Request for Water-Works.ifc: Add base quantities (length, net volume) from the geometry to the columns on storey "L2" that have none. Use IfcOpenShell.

First a look at what the model holds.

```python
import ifcopenshell
import ifcopenshell.util.element
import ifcopenshell.util.unit

model = ifcopenshell.open("Water-Works.ifc")
print(model.schema)
for unit_type in ("LENGTHUNIT", "AREAUNIT", "VOLUMEUNIT"):
    print(unit_type, ifcopenshell.util.unit.calculate_unit_scale(model, unit_type))
storey = next(s for s in model.by_type("IfcBuildingStorey") if s.Name == "L2")
columns = [e for e in ifcopenshell.util.element.get_decomposition(storey) if e.is_a("IfcColumn")]
for e in sorted(columns, key=lambda e: e.id()):
    print(e.id(), e.is_a(), e.Name, list(ifcopenshell.util.element.get_psets(e, qtos_only=True)), sep=" | ")
```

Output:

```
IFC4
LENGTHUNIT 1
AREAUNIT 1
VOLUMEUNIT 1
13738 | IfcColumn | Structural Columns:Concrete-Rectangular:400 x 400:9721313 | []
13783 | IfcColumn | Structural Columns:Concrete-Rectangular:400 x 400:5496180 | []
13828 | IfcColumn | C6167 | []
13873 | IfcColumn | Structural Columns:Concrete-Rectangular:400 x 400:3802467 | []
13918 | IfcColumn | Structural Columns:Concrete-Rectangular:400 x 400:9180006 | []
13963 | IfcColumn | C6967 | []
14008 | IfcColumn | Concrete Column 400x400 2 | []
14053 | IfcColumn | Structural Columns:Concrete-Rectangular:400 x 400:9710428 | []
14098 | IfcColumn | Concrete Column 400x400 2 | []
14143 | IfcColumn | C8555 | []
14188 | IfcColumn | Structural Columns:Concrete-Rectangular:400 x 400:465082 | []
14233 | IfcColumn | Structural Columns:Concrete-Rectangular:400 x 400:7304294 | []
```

```python
import ifcopenshell
import ifcopenshell.api.pset
import ifcopenshell.geom
import ifcopenshell.util.element
import ifcopenshell.util.shape
import ifcopenshell.util.unit

model = ifcopenshell.open("Water-Works.ifc")
unit_scale = ifcopenshell.util.unit.calculate_unit_scale(model)
volume_scale = ifcopenshell.util.unit.calculate_unit_scale(model, "VOLUMEUNIT")
settings = ifcopenshell.geom.settings()

storey = next(s for s in model.by_type("IfcBuildingStorey") if s.Name == "L2")
columns = [e for e in ifcopenshell.util.element.get_decomposition(storey) if e.is_a("IfcColumn")]

for e in sorted(columns, key=lambda e: e.id()):
    if ifcopenshell.util.element.get_psets(e, qtos_only=True, should_inherit=False):
        continue
    # Geometry comes back in metres, in the element's own axes.
    shape = ifcopenshell.geom.create_shape(settings, e)
    values = {
        "Length": ifcopenshell.util.shape.get_z(shape.geometry) / unit_scale,
        "NetVolume": ifcopenshell.util.shape.get_volume(shape.geometry) / volume_scale,
    }
    qto = ifcopenshell.api.pset.add_qto(model, product=e, name="Qto_ColumnBaseQuantities")
    ifcopenshell.api.pset.edit_qto(model, qto=qto, properties=values)
    print(e.id(), {k: round(v, 3) for k, v in values.items()})

model.write("Water-Works_updated.ifc")
```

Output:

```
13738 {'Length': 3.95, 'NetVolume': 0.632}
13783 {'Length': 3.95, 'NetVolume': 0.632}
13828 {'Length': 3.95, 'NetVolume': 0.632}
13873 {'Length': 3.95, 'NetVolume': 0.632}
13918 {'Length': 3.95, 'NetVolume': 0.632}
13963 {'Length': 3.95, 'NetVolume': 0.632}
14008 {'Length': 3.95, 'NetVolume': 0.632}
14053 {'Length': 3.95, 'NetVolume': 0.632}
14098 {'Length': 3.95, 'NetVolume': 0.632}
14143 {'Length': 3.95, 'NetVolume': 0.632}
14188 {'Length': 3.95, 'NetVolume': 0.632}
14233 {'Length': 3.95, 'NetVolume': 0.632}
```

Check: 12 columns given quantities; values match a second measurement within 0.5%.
